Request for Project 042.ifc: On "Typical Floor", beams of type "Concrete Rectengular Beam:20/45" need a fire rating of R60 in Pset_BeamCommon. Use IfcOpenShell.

First a look at what the model holds.

```python
import ifcopenshell
import ifcopenshell.util.element

model = ifcopenshell.open("Project 042.ifc")
print(model.schema)
storey = next(s for s in model.by_type("IfcBuildingStorey") if s.Name == "Typical Floor")
beams = [e for e in ifcopenshell.util.element.get_decomposition(storey) if e.is_a("IfcBeam")]
seen = {}
for e in beams:
    element_type = ifcopenshell.util.element.get_type(e)
    key = (element_type.Name if element_type != e and element_type else None, ifcopenshell.util.element.get_pset(e, "Pset_BeamCommon", "FireRating"))
    seen[key] = seen.get(key, 0) + 1
for (name, value), count in sorted(seen.items(), key=str):
    print(count, "x", name, "|", value)
```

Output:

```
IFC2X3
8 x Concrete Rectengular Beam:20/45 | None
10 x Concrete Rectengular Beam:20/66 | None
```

```python
import ifcopenshell
import ifcopenshell.api.pset
import ifcopenshell.util.element

model = ifcopenshell.open("Project 042.ifc")

storey = next(s for s in model.by_type("IfcBuildingStorey") if s.Name == "Typical Floor")
beams = [e for e in ifcopenshell.util.element.get_decomposition(storey) if e.is_a("IfcBeam")]

count = 0
for e in beams:
    element_type = ifcopenshell.util.element.get_type(e)
    if element_type in (None, e) or element_type.Name != "Concrete Rectengular Beam:20/45":
        continue
    # add_pset returns the element's existing set when there is one.
    pset = ifcopenshell.api.pset.add_pset(model, product=e, name="Pset_BeamCommon")
    ifcopenshell.api.pset.edit_pset(model, pset=pset, properties={"FireRating": "R60"})
    count += 1

print(count, "beams updated")

model.write("Project 042_updated.ifc")
```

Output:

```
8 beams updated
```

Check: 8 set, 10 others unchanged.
